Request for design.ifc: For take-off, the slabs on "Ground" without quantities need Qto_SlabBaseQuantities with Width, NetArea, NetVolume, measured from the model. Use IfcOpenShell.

First a look at what the model holds.

```python
import ifcopenshell
import ifcopenshell.util.element
import ifcopenshell.util.unit

model = ifcopenshell.open("design.ifc")
print(model.schema)
for unit_type in ("LENGTHUNIT", "AREAUNIT", "VOLUMEUNIT"):
    print(unit_type, ifcopenshell.util.unit.calculate_unit_scale(model, unit_type))
storey = next(s for s in model.by_type("IfcBuildingStorey") if s.Name == "Ground")
slabs = [e for e in ifcopenshell.util.element.get_decomposition(storey) if e.is_a("IfcSlab")]
for e in sorted(slabs, key=lambda e: e.id()):
    print(e.id(), e.is_a(), e.Name, list(ifcopenshell.util.element.get_psets(e, qtos_only=True)), sep=" | ")
```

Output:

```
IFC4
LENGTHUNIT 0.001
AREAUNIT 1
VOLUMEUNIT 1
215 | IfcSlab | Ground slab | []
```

```python
import ifcopenshell
import ifcopenshell.api.pset
import ifcopenshell.geom
import ifcopenshell.util.element
import ifcopenshell.util.shape
import ifcopenshell.util.unit

model = ifcopenshell.open("design.ifc")
unit_scale = ifcopenshell.util.unit.calculate_unit_scale(model)
area_scale = ifcopenshell.util.unit.calculate_unit_scale(model, "AREAUNIT")
volume_scale = ifcopenshell.util.unit.calculate_unit_scale(model, "VOLUMEUNIT")
settings = ifcopenshell.geom.settings()

storey = next(s for s in model.by_type("IfcBuildingStorey") if s.Name == "Ground")
slabs = [e for e in ifcopenshell.util.element.get_decomposition(storey) if e.is_a("IfcSlab")]

for e in sorted(slabs, key=lambda e: e.id()):
    if ifcopenshell.util.element.get_psets(e, qtos_only=True, should_inherit=False):
        continue
    # Geometry comes back in metres, in the element's own axes.
    shape = ifcopenshell.geom.create_shape(settings, e)
    values = {
        "Width": ifcopenshell.util.shape.get_z(shape.geometry) / unit_scale,
        "NetArea": ifcopenshell.util.shape.get_footprint_area(shape.geometry) / area_scale,
        "NetVolume": ifcopenshell.util.shape.get_volume(shape.geometry) / volume_scale,
    }
    qto = ifcopenshell.api.pset.add_qto(model, product=e, name="Qto_SlabBaseQuantities")
    ifcopenshell.api.pset.edit_qto(model, qto=qto, properties=values)
    print(e.id(), {k: round(v, 3) for k, v in values.items()})

model.write("design_rev.ifc")
```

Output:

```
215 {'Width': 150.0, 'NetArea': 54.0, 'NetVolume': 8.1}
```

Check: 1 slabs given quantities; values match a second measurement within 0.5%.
